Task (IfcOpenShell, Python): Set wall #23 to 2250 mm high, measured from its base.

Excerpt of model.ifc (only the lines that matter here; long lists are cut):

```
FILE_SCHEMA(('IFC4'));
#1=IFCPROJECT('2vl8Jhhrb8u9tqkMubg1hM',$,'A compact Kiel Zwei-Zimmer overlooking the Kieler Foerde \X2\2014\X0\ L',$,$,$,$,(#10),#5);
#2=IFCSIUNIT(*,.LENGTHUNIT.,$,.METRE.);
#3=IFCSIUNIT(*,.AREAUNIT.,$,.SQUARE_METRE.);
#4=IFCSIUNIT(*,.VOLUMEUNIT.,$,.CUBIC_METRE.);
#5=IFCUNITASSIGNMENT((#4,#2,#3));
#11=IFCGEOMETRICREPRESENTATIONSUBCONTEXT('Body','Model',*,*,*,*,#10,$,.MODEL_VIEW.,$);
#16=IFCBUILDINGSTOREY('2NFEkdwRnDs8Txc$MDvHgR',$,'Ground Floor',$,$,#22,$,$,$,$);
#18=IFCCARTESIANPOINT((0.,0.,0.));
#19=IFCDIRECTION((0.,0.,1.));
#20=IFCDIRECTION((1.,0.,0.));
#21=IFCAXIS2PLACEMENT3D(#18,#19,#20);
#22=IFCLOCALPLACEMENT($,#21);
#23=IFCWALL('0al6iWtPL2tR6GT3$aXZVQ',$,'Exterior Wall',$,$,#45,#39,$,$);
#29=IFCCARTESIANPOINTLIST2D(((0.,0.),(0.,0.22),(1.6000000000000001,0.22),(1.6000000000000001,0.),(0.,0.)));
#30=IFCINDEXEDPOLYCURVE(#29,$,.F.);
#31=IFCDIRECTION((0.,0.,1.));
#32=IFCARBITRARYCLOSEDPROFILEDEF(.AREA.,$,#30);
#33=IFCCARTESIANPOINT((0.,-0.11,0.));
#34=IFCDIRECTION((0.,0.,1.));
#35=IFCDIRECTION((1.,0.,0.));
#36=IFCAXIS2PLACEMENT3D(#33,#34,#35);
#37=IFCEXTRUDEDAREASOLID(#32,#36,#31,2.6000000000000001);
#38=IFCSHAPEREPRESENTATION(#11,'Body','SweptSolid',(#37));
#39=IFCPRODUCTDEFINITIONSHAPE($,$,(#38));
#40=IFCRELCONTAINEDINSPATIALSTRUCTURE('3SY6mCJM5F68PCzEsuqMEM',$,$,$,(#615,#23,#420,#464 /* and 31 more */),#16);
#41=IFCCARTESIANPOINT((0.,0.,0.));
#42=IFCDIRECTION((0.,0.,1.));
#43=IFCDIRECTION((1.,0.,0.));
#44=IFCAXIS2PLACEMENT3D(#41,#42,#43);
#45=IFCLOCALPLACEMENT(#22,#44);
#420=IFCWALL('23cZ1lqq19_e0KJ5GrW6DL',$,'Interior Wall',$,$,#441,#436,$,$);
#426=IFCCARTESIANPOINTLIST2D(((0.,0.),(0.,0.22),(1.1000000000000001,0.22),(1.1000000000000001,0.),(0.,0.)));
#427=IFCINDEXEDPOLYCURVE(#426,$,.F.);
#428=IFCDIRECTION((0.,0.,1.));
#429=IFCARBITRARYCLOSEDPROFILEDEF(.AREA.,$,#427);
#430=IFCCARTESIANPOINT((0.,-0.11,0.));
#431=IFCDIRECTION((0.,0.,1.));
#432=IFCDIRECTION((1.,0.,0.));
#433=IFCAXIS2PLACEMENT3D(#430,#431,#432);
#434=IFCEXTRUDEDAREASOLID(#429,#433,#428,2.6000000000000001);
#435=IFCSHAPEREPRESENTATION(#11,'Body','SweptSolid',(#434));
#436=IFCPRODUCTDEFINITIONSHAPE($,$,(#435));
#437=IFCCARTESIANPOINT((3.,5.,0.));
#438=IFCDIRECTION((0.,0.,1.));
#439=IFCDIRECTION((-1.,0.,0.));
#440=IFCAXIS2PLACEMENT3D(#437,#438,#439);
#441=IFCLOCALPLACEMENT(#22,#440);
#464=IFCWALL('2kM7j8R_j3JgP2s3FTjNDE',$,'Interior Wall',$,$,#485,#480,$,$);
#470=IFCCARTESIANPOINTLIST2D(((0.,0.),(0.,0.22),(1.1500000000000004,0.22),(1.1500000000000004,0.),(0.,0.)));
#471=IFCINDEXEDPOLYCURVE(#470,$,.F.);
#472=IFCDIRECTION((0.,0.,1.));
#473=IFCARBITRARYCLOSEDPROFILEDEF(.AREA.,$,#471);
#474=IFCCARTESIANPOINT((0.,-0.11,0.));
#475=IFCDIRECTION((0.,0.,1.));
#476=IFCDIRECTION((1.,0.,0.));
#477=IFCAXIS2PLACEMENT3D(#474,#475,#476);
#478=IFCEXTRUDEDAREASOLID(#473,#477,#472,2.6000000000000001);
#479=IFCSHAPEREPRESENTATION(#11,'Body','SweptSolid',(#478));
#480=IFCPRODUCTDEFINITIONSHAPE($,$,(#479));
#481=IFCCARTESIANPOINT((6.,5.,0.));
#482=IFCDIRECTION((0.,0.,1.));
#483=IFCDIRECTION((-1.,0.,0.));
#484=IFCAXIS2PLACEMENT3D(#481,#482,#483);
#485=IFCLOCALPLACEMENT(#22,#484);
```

```python
import ifcopenshell
import ifcopenshell.geom
import ifcopenshell.util.representation
import ifcopenshell.util.shape
import ifcopenshell.util.unit

model = ifcopenshell.open("model.ifc")
unit_scale = ifcopenshell.util.unit.calculate_unit_scale(model)
settings = ifcopenshell.geom.settings()


def volume(element):
    """Net volume in cubic metres, openings subtracted."""
    shape = ifcopenshell.geom.create_shape(settings, element)
    return ifcopenshell.util.shape.get_volume(shape.geometry)


wall = model.by_guid("0al6iWtPL2tR6GT3$aXZVQ")
before = volume(wall)

body = ifcopenshell.util.representation.get_representation(wall, "Model", "Body")
solid = body.Items[0]
old_height = solid.Depth
solid.Depth = 2.25 / unit_scale
after = volume(wall)

print(f"height {old_height:g} -> {solid.Depth:g}, volume {before:.3f} -> {after:.3f} m3")

model.write("model_edited.ifc")
```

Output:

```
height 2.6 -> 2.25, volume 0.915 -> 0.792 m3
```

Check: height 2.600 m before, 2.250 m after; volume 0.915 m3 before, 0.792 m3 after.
